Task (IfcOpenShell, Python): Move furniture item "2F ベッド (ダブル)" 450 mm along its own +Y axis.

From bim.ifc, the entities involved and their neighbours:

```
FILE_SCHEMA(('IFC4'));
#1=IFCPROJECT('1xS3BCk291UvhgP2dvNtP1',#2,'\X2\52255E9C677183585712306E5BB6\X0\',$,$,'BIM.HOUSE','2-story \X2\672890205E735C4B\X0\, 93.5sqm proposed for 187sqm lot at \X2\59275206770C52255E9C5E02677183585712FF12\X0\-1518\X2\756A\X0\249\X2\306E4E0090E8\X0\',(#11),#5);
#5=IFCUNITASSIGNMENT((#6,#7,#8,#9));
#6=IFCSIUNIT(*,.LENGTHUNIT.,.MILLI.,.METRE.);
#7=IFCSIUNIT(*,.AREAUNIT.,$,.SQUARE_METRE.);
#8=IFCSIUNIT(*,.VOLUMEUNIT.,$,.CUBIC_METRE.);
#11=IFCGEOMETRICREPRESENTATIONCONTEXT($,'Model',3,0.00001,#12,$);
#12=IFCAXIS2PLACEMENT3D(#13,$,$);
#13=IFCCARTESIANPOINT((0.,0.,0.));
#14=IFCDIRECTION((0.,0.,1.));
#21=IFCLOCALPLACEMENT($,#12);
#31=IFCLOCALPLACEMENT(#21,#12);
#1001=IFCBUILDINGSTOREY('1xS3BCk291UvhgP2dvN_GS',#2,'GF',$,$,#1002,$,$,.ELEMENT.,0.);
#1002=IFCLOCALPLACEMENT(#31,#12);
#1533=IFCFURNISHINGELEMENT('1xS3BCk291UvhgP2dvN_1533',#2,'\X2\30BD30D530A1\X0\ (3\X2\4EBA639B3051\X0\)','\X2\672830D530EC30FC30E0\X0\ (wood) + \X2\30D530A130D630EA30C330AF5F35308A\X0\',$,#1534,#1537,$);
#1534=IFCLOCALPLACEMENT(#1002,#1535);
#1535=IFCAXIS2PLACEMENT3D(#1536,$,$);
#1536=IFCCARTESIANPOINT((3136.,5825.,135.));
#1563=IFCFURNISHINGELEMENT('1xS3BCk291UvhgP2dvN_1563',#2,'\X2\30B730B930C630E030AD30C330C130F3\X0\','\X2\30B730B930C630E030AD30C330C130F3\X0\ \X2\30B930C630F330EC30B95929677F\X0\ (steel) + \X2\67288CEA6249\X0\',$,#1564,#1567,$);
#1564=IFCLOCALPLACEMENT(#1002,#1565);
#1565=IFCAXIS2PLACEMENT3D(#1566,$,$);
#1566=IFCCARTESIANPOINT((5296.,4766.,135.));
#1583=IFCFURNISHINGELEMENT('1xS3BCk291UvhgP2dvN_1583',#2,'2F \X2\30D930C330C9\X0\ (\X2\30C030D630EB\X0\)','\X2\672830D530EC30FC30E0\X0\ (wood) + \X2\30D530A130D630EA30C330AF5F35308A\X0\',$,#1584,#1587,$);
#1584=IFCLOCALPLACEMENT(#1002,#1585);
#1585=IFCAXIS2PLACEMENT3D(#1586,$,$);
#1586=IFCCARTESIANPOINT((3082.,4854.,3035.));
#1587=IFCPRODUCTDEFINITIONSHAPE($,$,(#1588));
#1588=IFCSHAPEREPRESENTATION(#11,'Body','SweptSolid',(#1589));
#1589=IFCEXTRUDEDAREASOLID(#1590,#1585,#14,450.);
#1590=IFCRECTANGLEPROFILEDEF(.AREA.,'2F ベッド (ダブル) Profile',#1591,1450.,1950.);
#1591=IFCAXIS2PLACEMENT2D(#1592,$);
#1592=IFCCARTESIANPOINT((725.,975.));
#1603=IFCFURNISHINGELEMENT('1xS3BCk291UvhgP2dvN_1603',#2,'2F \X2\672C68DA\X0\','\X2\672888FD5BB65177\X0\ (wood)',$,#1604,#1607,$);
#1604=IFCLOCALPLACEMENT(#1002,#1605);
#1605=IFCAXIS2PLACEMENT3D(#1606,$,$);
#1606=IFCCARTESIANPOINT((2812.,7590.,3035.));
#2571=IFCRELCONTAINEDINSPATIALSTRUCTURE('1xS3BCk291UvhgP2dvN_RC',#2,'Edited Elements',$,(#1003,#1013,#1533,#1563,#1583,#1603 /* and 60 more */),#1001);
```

```python
import ifcopenshell
import ifcopenshell.api.geometry
import ifcopenshell.util.placement
import ifcopenshell.util.unit

model = ifcopenshell.open("bim.ifc")
unit_scale = ifcopenshell.util.unit.calculate_unit_scale(model)

item = model.by_guid("1xS3BCk291UvhgP2dvN_1583")
matrix = ifcopenshell.util.placement.get_local_placement(item.ObjectPlacement)
matrix[:3, 3] += matrix[:3, 1] * 0.45 / unit_scale
ifcopenshell.api.geometry.edit_object_placement(model, product=item, matrix=matrix, is_si=False)

print(ifcopenshell.util.placement.get_local_placement(item.ObjectPlacement).round(3) + 0.0)

model.write("bim_updated.ifc")
```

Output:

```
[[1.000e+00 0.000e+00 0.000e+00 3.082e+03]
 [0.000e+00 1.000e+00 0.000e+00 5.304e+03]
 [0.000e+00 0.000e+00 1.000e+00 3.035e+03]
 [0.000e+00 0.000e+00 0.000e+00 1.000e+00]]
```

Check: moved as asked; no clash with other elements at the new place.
